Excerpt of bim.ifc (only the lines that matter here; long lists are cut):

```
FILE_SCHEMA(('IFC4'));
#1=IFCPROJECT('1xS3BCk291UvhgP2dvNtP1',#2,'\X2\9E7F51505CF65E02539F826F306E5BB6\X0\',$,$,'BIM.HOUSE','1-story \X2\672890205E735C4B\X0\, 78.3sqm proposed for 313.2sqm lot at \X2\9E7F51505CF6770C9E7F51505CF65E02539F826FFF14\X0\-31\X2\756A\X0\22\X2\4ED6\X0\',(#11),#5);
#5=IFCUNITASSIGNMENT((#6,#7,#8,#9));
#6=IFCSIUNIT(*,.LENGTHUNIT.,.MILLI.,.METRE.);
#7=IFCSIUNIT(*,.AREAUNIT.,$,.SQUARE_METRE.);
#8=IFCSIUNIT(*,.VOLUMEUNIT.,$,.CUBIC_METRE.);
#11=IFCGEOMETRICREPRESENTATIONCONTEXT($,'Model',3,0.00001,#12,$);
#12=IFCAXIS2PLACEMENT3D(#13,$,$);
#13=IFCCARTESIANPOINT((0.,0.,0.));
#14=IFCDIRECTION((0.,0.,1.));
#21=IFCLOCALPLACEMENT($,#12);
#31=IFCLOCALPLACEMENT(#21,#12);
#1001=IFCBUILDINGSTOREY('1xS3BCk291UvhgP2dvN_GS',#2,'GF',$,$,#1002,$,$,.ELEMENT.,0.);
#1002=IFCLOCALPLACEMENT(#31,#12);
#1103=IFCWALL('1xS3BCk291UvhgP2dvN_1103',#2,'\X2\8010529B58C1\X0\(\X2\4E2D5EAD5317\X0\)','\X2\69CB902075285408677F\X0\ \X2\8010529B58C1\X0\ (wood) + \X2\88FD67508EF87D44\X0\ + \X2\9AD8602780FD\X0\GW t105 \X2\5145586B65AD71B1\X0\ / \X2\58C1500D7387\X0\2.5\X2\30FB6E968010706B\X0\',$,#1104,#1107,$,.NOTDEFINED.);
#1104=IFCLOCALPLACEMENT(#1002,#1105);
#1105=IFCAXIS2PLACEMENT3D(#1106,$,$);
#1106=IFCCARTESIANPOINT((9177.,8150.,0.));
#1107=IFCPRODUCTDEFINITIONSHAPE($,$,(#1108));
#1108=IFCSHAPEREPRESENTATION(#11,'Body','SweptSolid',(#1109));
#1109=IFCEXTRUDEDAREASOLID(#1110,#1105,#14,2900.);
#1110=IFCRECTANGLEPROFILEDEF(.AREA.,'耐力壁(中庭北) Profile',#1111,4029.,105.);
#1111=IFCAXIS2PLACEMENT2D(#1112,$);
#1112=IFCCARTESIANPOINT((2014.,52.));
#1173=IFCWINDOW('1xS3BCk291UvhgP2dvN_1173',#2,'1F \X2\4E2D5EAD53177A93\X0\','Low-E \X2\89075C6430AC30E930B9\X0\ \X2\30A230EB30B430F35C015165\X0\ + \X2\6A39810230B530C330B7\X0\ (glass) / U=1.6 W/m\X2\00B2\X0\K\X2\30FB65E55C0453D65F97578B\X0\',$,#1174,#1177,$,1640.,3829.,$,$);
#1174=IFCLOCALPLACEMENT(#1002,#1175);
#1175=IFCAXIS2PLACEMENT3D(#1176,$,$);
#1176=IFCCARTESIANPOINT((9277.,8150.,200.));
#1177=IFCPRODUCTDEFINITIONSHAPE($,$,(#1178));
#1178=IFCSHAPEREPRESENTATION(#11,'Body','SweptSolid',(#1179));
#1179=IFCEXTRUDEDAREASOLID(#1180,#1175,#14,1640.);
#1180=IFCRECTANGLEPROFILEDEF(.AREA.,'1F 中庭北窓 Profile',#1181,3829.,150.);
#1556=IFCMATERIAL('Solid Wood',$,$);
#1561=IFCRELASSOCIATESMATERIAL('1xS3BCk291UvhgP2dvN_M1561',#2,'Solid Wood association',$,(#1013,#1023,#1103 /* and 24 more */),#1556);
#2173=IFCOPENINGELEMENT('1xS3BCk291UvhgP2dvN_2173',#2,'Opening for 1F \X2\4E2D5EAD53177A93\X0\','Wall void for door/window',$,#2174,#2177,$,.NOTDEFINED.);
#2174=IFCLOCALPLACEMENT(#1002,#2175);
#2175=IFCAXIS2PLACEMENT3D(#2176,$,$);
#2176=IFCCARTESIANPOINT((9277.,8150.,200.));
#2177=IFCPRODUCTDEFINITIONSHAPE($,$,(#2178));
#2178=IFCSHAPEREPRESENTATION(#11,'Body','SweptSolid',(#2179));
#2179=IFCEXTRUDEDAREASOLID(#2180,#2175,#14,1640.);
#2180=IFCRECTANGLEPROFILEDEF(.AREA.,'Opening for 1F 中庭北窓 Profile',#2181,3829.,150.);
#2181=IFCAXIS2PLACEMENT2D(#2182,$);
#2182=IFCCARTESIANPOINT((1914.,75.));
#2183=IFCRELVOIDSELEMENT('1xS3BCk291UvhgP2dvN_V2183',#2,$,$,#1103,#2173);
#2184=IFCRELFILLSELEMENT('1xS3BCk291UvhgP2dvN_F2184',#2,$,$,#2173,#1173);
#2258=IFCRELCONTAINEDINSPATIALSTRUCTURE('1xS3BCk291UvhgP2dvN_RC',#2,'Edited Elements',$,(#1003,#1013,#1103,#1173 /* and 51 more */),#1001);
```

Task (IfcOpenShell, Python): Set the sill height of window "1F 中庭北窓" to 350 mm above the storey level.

```python
import numpy as np
import ifcopenshell
import ifcopenshell.api.geometry
import ifcopenshell.geom
import ifcopenshell.util.element
import ifcopenshell.util.placement
import ifcopenshell.util.shape
import ifcopenshell.util.unit

model = ifcopenshell.open("bim.ifc")
unit_scale = ifcopenshell.util.unit.calculate_unit_scale(model)

window = model.by_guid("1xS3BCk291UvhgP2dvN_1173")
opening = window.FillsVoids[0].RelatingOpeningElement
storey = ifcopenshell.util.element.get_container(window, ifc_class="IfcBuildingStorey")
level = ifcopenshell.util.placement.get_local_placement(storey.ObjectPlacement)[2, 3]

# The opening's origin need not be at the sill, so measure its lowest point.
shape = ifcopenshell.geom.create_shape(ifcopenshell.geom.settings(), opening)
bottom = ifcopenshell.util.shape.get_shape_bottom_elevation(shape, shape.geometry) / unit_scale
dz = level + 350.0 - bottom

shift = np.array([0.0, 0.0, dz])
# The window is not placed relative to its opening, so move both.
for product in (opening, window):
    matrix = ifcopenshell.util.placement.get_local_placement(product.ObjectPlacement)
    matrix[:3, 3] += shift
    ifcopenshell.api.geometry.edit_object_placement(model, product=product, matrix=matrix, is_si=False)

print(f"moved by {dz * unit_scale:+.3f} m")

model.write("bim_updated.ifc")
```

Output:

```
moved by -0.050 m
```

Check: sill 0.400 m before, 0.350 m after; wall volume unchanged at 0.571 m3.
